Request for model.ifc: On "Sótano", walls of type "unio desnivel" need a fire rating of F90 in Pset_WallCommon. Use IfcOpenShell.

First a look at what the model holds.

```python
import ifcopenshell
import ifcopenshell.util.element

model = ifcopenshell.open("model.ifc")
print(model.schema)
storey = next(s for s in model.by_type("IfcBuildingStorey") if s.Name == "Sótano")
walls = [e for e in ifcopenshell.util.element.get_decomposition(storey) if e.is_a("IfcWall")]
seen = {}
for e in walls:
    element_type = ifcopenshell.util.element.get_type(e)
    key = (element_type.Name if element_type != e and element_type else None, ifcopenshell.util.element.get_pset(e, "Pset_WallCommon", "FireRating"))
    seen[key] = seen.get(key, 0) + 1
for (name, value), count in sorted(seen.items(), key=str):
    print(count, "x", name, "|", value)
```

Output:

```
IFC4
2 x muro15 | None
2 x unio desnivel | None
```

```python
import ifcopenshell
import ifcopenshell.api.pset
import ifcopenshell.util.element

model = ifcopenshell.open("model.ifc")

storey = next(s for s in model.by_type("IfcBuildingStorey") if s.Name == "Sótano")
walls = [e for e in ifcopenshell.util.element.get_decomposition(storey) if e.is_a("IfcWall")]

count = 0
for e in walls:
    element_type = ifcopenshell.util.element.get_type(e)
    if element_type in (None, e) or element_type.Name != "unio desnivel":
        continue
    # add_pset returns the element's existing set when there is one.
    pset = ifcopenshell.api.pset.add_pset(model, product=e, name="Pset_WallCommon")
    ifcopenshell.api.pset.edit_pset(model, pset=pset, properties={"FireRating": "F90"})
    count += 1

print(count, "walls updated")

model.write("model_updated.ifc")
```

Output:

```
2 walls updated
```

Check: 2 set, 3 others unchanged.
